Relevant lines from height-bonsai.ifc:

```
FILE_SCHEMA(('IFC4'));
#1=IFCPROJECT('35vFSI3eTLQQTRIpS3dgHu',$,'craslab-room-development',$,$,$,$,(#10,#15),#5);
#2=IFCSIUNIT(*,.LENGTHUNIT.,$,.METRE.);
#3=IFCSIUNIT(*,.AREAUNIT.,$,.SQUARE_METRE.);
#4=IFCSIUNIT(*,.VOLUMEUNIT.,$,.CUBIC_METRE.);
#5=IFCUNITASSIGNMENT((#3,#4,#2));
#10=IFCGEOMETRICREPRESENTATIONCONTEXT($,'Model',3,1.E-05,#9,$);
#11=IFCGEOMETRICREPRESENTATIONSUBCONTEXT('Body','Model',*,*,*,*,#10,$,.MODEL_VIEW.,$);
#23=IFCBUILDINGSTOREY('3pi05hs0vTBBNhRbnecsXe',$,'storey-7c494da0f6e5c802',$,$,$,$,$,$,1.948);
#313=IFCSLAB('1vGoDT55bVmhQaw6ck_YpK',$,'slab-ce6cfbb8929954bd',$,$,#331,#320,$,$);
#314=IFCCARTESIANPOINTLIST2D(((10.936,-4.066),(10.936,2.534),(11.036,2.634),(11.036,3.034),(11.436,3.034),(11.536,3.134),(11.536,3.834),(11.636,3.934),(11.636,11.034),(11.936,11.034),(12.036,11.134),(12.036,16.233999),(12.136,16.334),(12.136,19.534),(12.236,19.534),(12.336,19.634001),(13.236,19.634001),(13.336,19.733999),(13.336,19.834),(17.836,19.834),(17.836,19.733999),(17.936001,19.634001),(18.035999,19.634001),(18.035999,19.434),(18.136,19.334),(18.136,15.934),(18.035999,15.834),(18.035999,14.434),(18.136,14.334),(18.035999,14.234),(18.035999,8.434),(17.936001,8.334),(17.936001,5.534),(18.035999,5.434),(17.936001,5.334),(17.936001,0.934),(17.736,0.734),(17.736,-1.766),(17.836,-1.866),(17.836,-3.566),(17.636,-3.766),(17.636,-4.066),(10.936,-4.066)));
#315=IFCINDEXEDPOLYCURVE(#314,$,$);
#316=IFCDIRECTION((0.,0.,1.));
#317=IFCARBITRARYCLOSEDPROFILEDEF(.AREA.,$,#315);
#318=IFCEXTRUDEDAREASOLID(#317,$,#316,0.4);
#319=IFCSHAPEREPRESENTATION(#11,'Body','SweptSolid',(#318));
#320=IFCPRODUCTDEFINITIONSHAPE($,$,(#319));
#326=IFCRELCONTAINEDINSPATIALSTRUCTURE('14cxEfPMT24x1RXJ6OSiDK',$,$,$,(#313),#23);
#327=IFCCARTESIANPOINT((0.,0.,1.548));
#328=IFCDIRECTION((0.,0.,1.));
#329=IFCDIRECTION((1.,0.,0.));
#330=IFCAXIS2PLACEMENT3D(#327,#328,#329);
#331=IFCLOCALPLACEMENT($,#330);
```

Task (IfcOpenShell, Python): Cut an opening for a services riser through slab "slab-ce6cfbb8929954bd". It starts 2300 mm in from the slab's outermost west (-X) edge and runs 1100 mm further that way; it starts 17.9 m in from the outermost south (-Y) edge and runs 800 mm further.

```python
import numpy as np
import ifcopenshell
import ifcopenshell.api.feature
import ifcopenshell.api.geometry
import ifcopenshell.api.root
import ifcopenshell.geom
import ifcopenshell.util.placement
import ifcopenshell.util.representation
import ifcopenshell.util.shape
import ifcopenshell.util.unit

model = ifcopenshell.open("height-bonsai.ifc")
unit_scale = ifcopenshell.util.unit.calculate_unit_scale(model)
settings = ifcopenshell.geom.settings()


def volume(element):
    """Net volume in cubic metres, openings subtracted."""
    shape = ifcopenshell.geom.create_shape(settings, element)
    return ifcopenshell.util.shape.get_volume(shape.geometry)


slab = model.by_id(313)
before = volume(slab)

# Extent in the slab's own axes, in metres. The edges named are its -X and -Y sides.
slab_shape = ifcopenshell.geom.create_shape(settings, slab)
vertices = ifcopenshell.util.shape.get_vertices(slab_shape.geometry)
x_min, y_min, bottom = vertices.min(axis=0)
top = vertices[:, 2].max()

opening = ifcopenshell.api.root.create_entity(model, ifc_class="IfcOpeningElement", name="Services riser opening", predefined_type="OPENING")
context = ifcopenshell.util.representation.get_context(model, "Model", "Body", "MODEL_VIEW")
width, depth = 1.1, 0.8
outline = [(0.0, 0.0), (width, 0.0), (width, depth), (0.0, depth), (0.0, 0.0)]
# Overshoot both faces by 50 mm so the cut is clean.
shape = ifcopenshell.api.geometry.add_slab_representation(
    model, context=context, depth=top - bottom + 0.1, polyline=outline
)
ifcopenshell.api.geometry.assign_representation(model, product=opening, representation=shape)

matrix = ifcopenshell.util.placement.get_local_placement(slab.ObjectPlacement)
matrix[:, 3] = matrix @ np.append(np.array([x_min + 2.3, y_min + 17.9, bottom - 0.05]) / unit_scale, 1.0)
ifcopenshell.api.geometry.edit_object_placement(model, product=opening, matrix=matrix, is_si=False)
ifcopenshell.api.feature.add_feature(model, feature=opening, element=slab)

after = volume(slab)

print(f"slab volume {before:.3f} -> {after:.3f} m3")

model.write("height-bonsai_edited.ifc")
```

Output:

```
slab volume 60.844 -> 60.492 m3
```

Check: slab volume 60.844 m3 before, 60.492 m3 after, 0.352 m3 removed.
